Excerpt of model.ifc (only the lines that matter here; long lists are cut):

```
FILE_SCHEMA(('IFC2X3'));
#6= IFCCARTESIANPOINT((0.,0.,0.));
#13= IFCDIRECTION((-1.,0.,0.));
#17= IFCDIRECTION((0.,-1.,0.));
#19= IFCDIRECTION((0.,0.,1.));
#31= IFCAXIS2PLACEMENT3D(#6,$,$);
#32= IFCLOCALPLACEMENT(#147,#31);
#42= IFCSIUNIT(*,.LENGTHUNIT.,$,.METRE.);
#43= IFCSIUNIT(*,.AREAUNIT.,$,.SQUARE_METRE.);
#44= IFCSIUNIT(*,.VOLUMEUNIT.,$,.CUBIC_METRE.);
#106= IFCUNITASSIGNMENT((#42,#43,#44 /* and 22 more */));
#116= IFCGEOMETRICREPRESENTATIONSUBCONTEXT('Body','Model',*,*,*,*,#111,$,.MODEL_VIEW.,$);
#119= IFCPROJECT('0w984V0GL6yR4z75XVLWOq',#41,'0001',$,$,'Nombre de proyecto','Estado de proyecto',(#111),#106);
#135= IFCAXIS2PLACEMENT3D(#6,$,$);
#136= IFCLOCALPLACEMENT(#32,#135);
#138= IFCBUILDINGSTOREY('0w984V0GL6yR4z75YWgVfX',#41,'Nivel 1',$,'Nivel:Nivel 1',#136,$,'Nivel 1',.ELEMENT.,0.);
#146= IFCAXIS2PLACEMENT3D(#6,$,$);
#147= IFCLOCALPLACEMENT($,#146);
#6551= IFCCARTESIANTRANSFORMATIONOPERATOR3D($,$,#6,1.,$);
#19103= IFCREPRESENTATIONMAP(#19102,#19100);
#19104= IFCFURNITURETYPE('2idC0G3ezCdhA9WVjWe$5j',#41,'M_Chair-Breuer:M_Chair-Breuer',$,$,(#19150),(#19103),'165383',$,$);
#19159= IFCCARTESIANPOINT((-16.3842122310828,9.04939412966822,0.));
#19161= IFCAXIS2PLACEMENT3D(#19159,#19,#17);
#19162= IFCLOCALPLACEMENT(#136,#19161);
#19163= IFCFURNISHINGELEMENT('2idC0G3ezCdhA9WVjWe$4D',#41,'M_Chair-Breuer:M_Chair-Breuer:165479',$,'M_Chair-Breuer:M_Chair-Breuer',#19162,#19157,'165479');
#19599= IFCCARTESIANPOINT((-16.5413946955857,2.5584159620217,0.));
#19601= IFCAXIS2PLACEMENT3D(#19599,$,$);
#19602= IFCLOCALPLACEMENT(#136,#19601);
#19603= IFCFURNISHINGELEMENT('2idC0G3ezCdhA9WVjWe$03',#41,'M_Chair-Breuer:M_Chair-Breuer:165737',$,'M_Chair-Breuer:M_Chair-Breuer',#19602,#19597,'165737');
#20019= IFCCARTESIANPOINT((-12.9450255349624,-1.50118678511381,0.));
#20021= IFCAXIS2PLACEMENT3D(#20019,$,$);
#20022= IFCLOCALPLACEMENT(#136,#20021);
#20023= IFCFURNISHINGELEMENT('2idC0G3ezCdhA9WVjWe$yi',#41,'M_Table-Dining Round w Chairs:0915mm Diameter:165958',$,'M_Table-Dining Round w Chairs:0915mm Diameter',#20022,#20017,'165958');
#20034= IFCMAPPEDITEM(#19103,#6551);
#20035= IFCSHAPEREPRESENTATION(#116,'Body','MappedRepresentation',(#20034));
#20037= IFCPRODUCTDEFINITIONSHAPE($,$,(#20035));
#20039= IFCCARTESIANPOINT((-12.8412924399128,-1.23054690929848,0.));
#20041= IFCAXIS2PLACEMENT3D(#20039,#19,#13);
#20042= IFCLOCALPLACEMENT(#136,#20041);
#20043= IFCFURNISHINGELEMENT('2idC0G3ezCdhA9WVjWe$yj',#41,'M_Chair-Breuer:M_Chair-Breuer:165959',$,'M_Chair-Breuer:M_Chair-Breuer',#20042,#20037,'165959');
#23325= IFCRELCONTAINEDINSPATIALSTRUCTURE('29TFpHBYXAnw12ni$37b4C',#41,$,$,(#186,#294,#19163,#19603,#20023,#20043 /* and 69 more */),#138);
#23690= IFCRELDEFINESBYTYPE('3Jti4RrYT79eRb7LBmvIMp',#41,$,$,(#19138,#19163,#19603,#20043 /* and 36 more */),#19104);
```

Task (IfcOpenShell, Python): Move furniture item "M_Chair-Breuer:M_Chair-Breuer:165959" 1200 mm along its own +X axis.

```python
import ifcopenshell
import ifcopenshell.api.geometry
import ifcopenshell.util.placement
import ifcopenshell.util.unit

model = ifcopenshell.open("model.ifc")
unit_scale = ifcopenshell.util.unit.calculate_unit_scale(model)

item = model.by_guid("2idC0G3ezCdhA9WVjWe$yj")
matrix = ifcopenshell.util.placement.get_local_placement(item.ObjectPlacement)
matrix[:3, 3] += matrix[:3, 0] * 1.2 / unit_scale
ifcopenshell.api.geometry.edit_object_placement(model, product=item, matrix=matrix, is_si=False)

print(ifcopenshell.util.placement.get_local_placement(item.ObjectPlacement).round(3) + 0.0)

model.write("model-out.ifc")
```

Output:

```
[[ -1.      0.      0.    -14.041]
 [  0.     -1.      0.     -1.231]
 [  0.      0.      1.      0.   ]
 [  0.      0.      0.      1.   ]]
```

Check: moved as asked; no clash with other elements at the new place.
